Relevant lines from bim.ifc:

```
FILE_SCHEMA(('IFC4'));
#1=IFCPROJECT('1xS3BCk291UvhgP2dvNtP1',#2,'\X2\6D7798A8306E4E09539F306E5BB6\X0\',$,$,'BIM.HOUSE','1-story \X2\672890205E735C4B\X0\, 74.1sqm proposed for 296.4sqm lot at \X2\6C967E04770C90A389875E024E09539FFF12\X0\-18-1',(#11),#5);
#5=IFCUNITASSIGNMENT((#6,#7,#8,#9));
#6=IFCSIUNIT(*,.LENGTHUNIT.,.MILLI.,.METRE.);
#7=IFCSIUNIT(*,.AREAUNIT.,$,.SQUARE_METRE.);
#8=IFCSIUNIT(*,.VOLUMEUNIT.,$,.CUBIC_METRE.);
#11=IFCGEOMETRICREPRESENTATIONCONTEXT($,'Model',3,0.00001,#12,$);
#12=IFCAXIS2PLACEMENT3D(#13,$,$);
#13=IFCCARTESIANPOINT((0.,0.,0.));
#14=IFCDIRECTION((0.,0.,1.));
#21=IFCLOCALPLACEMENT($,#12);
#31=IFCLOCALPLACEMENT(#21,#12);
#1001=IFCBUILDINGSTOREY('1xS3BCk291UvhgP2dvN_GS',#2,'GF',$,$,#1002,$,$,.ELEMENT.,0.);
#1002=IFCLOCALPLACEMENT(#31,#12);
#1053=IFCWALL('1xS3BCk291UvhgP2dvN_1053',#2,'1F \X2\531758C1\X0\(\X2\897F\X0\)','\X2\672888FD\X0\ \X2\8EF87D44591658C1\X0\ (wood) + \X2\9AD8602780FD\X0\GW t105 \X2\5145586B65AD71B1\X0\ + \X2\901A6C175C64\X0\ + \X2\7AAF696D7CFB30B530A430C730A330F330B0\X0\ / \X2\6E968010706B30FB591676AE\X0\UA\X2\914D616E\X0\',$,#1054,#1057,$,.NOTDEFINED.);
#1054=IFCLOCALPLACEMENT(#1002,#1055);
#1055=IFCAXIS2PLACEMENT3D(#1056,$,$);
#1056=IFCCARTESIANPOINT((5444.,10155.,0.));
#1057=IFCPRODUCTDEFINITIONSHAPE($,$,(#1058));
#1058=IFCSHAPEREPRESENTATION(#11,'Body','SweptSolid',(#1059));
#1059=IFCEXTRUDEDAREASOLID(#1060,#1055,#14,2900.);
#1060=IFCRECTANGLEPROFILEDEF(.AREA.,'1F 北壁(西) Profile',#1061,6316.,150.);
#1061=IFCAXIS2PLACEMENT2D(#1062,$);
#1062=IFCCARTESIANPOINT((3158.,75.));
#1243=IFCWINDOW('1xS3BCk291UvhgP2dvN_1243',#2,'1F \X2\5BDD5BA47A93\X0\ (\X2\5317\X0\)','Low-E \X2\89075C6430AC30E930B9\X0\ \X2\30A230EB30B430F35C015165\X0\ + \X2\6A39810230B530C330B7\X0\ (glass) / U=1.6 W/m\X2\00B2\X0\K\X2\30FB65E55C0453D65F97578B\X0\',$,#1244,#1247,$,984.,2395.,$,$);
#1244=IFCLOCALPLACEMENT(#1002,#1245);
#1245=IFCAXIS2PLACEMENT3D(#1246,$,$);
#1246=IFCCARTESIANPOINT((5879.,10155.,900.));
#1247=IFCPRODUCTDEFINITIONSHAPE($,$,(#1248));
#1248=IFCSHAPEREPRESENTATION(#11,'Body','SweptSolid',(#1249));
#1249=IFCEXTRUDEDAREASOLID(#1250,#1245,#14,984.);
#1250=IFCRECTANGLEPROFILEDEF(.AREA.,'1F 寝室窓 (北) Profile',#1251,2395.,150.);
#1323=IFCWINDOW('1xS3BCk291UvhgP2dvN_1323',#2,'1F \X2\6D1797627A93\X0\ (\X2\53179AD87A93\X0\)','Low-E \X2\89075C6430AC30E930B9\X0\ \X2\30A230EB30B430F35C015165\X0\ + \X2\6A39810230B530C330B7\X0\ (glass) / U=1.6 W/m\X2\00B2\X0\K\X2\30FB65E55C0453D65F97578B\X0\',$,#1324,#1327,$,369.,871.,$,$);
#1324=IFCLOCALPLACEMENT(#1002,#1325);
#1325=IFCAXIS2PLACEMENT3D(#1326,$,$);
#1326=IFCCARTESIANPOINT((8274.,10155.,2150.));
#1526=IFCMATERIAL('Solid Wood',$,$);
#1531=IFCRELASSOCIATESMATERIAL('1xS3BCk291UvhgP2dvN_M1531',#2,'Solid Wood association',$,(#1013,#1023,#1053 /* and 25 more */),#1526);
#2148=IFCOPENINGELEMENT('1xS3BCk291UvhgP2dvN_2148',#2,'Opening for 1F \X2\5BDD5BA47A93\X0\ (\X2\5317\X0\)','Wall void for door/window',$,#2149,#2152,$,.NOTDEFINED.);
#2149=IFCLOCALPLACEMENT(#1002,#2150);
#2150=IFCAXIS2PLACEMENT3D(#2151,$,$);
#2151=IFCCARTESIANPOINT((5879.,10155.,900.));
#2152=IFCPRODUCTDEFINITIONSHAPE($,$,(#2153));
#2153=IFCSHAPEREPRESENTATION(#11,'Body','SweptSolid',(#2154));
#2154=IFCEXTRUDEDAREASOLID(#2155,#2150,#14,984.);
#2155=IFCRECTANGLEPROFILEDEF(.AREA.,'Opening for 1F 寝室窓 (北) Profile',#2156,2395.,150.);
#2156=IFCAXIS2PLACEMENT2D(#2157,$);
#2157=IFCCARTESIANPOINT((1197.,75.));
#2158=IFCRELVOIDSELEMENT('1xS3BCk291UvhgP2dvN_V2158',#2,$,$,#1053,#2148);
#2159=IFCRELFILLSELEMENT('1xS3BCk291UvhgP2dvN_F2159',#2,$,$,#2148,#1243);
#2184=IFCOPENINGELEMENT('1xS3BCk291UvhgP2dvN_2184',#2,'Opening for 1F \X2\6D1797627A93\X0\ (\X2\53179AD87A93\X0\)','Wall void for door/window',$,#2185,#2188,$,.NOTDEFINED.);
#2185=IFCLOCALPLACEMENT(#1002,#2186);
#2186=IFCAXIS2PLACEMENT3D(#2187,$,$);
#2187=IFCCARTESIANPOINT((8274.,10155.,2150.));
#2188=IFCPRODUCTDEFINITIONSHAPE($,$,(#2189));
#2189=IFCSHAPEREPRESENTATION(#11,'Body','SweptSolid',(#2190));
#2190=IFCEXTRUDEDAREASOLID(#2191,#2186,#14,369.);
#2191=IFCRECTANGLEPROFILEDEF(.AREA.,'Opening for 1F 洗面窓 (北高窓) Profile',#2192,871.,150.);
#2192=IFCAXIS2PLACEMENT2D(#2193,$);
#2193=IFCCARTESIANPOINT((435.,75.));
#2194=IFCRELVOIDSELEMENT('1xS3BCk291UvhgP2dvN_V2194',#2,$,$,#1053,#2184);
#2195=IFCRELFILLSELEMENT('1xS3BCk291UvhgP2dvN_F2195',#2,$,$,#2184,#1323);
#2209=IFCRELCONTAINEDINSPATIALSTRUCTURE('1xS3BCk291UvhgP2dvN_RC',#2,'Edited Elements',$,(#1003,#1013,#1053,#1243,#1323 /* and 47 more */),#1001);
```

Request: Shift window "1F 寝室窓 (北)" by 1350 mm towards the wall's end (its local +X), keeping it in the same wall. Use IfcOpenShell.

```python
import ifcopenshell
import ifcopenshell.api.geometry
import ifcopenshell.util.placement
import ifcopenshell.util.unit

model = ifcopenshell.open("bim.ifc")
unit_scale = ifcopenshell.util.unit.calculate_unit_scale(model)

window = model.by_guid("1xS3BCk291UvhgP2dvN_1243")
opening = window.FillsVoids[0].RelatingOpeningElement
wall = opening.VoidsElements[0].RelatingBuildingElement

wall_matrix = ifcopenshell.util.placement.get_local_placement(wall.ObjectPlacement)
shift = wall_matrix[:3, 0] * 1.35 / unit_scale
before = ifcopenshell.util.placement.get_local_placement(window.ObjectPlacement)[:3, 3].copy()

# The window is not placed relative to its opening, so move both.
for product in (opening, window):
    matrix = ifcopenshell.util.placement.get_local_placement(product.ObjectPlacement)
    matrix[:3, 3] += shift
    ifcopenshell.api.geometry.edit_object_placement(model, product=product, matrix=matrix, is_si=False)

after = ifcopenshell.util.placement.get_local_placement(window.ObjectPlacement)[:3, 3]
print("window moved by", (after - before).round(3) + 0.0)

model.write("bim_rev.ifc")
```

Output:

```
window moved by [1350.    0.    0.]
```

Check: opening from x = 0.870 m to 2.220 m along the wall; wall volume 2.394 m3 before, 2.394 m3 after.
